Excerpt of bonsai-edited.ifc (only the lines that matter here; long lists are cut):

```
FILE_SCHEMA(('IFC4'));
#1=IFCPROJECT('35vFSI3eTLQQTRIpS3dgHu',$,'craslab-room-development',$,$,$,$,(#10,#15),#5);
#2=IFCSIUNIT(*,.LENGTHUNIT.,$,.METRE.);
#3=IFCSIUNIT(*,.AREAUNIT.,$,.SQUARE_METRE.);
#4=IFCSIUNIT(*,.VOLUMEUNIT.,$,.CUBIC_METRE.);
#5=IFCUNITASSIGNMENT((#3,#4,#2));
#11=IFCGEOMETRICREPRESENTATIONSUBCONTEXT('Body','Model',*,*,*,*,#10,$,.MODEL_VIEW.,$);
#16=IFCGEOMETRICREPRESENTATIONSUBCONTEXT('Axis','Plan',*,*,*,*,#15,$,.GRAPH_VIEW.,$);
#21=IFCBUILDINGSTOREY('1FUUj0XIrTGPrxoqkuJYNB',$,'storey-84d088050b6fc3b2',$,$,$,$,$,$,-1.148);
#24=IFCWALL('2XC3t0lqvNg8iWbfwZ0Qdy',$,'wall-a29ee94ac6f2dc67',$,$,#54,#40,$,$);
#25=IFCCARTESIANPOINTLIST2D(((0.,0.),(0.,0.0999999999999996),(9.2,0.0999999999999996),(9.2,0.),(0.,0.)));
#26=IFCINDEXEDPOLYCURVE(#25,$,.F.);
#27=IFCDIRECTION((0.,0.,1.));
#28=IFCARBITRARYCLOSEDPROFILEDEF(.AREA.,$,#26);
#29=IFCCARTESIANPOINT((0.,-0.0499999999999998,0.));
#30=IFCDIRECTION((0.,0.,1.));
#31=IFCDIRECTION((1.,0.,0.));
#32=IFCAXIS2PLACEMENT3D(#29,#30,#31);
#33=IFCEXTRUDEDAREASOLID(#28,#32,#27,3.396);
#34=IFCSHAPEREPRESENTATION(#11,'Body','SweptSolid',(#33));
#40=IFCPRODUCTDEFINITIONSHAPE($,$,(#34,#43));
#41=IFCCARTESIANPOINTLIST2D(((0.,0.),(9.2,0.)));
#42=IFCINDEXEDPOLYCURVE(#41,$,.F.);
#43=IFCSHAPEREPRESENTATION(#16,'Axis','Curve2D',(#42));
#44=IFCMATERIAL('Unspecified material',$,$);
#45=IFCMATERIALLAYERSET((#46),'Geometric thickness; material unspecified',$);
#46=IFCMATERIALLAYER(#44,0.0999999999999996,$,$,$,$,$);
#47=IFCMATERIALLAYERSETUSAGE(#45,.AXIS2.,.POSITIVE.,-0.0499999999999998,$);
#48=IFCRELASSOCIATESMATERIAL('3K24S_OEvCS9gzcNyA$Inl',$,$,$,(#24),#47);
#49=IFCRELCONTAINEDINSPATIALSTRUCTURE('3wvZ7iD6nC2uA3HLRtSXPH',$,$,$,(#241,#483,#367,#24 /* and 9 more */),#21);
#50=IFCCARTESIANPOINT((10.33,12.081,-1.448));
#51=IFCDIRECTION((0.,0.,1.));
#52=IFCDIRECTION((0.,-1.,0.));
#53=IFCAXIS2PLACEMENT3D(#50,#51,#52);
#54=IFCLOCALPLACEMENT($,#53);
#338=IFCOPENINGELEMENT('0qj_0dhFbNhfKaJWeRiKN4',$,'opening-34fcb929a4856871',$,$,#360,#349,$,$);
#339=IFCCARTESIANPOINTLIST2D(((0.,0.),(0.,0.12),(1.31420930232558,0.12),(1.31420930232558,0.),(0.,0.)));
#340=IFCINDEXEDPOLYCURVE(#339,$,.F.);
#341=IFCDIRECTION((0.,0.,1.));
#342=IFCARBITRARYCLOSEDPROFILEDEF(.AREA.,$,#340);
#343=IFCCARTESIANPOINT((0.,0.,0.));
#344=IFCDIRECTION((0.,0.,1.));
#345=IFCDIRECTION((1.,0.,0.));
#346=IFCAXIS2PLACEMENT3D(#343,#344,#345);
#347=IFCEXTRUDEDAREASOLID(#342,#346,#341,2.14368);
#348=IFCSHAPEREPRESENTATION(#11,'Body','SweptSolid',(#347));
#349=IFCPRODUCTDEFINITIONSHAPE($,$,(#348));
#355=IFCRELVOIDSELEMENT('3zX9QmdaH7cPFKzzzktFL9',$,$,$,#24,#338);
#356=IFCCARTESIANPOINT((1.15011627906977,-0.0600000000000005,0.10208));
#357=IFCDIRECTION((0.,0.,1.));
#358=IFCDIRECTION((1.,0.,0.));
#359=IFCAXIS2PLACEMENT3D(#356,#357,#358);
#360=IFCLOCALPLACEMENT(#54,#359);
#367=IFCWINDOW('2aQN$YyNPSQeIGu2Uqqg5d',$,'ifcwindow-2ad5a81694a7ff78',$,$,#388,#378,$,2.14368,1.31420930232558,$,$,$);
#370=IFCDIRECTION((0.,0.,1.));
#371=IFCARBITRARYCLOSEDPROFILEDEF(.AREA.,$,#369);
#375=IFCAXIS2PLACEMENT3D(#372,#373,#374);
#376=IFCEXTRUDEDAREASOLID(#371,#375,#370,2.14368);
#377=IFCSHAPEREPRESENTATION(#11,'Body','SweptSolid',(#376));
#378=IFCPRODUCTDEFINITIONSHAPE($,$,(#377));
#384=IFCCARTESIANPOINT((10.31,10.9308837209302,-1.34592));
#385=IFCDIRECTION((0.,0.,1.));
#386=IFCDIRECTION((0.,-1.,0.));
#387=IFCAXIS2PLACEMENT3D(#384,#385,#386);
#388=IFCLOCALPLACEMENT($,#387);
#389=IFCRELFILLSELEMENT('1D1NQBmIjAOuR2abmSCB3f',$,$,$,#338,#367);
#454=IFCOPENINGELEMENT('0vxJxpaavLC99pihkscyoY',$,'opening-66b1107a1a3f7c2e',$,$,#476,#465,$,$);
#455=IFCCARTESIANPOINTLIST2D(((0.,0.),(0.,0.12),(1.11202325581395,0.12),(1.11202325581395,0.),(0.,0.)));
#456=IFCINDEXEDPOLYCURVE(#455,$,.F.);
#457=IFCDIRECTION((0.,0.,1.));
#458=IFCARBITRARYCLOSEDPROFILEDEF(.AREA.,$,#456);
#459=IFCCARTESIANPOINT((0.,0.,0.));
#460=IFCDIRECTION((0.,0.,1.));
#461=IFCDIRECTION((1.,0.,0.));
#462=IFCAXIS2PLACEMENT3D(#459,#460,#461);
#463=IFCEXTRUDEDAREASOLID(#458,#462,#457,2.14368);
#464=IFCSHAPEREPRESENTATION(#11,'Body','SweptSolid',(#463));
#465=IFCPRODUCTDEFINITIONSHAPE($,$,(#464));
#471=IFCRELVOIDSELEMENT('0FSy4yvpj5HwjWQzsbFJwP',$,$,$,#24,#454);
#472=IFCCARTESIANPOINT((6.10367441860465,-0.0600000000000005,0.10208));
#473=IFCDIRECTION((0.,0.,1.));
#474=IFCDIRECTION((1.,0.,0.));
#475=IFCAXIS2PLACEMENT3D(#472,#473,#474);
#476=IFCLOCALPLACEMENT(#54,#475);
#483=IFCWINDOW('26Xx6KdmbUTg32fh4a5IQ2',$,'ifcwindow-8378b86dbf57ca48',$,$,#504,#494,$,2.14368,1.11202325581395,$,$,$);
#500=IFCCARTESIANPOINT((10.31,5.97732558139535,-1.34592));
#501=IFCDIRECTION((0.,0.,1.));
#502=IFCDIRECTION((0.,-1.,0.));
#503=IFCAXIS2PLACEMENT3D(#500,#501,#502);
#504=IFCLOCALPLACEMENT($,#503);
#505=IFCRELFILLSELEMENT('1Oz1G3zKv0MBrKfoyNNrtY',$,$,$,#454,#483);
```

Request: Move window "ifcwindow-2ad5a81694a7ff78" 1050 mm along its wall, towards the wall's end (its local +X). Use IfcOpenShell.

```python
import ifcopenshell
import ifcopenshell.api.geometry
import ifcopenshell.util.placement
import ifcopenshell.util.unit

model = ifcopenshell.open("bonsai-edited.ifc")
unit_scale = ifcopenshell.util.unit.calculate_unit_scale(model)

window = model.by_id(367)
opening = window.FillsVoids[0].RelatingOpeningElement
wall = opening.VoidsElements[0].RelatingBuildingElement

wall_matrix = ifcopenshell.util.placement.get_local_placement(wall.ObjectPlacement)
shift = wall_matrix[:3, 0] * 1.05 / unit_scale
before = ifcopenshell.util.placement.get_local_placement(window.ObjectPlacement)[:3, 3].copy()

# The window is not placed relative to its opening, so move both.
for product in (opening, window):
    matrix = ifcopenshell.util.placement.get_local_placement(product.ObjectPlacement)
    matrix[:3, 3] += shift
    ifcopenshell.api.geometry.edit_object_placement(model, product=product, matrix=matrix, is_si=False)

after = ifcopenshell.util.placement.get_local_placement(window.ObjectPlacement)[:3, 3]
print("window moved by", (after - before).round(3) + 0.0)

model.write("bonsai-edited_updated.ifc")
```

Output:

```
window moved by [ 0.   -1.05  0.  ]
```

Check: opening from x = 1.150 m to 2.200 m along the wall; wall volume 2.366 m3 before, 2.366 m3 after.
